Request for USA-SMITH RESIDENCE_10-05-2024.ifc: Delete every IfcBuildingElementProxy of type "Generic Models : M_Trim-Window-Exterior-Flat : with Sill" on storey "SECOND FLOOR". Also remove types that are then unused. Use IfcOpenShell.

First a look at what the model holds.

```python
import ifcopenshell
import ifcopenshell.util.element

model = ifcopenshell.open("USA-SMITH RESIDENCE_10-05-2024.ifc")
print(model.schema)
storey = next(s for s in model.by_type("IfcBuildingStorey") if s.Name == "SECOND FLOOR")
proxies = [e for e in ifcopenshell.util.element.get_decomposition(storey) if e.is_a("IfcBuildingElementProxy")]
seen = {}
for e in proxies:
    element_type = ifcopenshell.util.element.get_type(e)
    name = element_type.Name if element_type not in (None, e) else None
    seen[name] = seen.get(name, 0) + 1
for name, count in sorted(seen.items(), key=str):
    print(count, "x", name)
```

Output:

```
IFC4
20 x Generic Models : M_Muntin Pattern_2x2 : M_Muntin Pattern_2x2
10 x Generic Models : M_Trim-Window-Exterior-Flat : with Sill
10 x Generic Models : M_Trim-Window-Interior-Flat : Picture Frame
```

```python
import ifcopenshell
import ifcopenshell.api.root
import ifcopenshell.util.element

model = ifcopenshell.open("USA-SMITH RESIDENCE_10-05-2024.ifc")

storey = next(s for s in model.by_type("IfcBuildingStorey") if s.Name == "SECOND FLOOR")
proxies = [e for e in ifcopenshell.util.element.get_decomposition(storey) if e.is_a("IfcBuildingElementProxy")]
targets = [e for e in proxies if (t := ifcopenshell.util.element.get_type(e)) not in (None, e) and t.Name == "Generic Models : M_Trim-Window-Exterior-Flat : with Sill"]
types = {ifcopenshell.util.element.get_type(e) for e in targets} - {None, *targets}

for e in targets:
    ifcopenshell.api.root.remove_product(model, product=e)
print(len(targets), "removed")

unused = [t for t in types if not ifcopenshell.util.element.get_types(t)]
for t in unused:
    ifcopenshell.api.root.remove_product(model, product=t)
print(len(unused), "unused types removed")

model.write("USA-SMITH RESIDENCE_10-05-2024_edited.ifc")
```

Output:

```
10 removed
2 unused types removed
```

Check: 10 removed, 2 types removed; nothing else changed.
